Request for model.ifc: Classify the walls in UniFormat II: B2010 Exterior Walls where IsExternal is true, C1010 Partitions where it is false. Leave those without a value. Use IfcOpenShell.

First a look at what the model holds.

```python
import ifcopenshell
import ifcopenshell.util.element

model = ifcopenshell.open("model.ifc")
print(model.schema)
print("classifications:", [c.Name for c in model.by_type("IfcClassification")])
values = [ifcopenshell.util.element.get_pset(e, "Pset_WallCommon", "IsExternal") for e in model.by_type("IfcWall")]
for value in (True, False, None):
    print("IsExternal", value, values.count(value))
```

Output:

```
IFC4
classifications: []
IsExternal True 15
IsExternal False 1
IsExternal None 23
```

```python
import ifcopenshell
import ifcopenshell.api.classification
import ifcopenshell.util.element

model = ifcopenshell.open("model.ifc")

system = ifcopenshell.api.classification.add_classification(model, classification="UniFormat II")

walls = model.by_type("IfcWall")
external = {e: ifcopenshell.util.element.get_pset(e, "Pset_WallCommon", "IsExternal") for e in walls}
for flag, code, name in ((True, "B2010", "Exterior Walls"), (False, "C1010", "Partitions")):
    products = [e for e in walls if external[e] is flag]
    ifcopenshell.api.classification.add_reference(
        model, products=products, classification=system, identification=code, name=name
    )
    print(code, len(products))

model.write("model_updated.ifc")
```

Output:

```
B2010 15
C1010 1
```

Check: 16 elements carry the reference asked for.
